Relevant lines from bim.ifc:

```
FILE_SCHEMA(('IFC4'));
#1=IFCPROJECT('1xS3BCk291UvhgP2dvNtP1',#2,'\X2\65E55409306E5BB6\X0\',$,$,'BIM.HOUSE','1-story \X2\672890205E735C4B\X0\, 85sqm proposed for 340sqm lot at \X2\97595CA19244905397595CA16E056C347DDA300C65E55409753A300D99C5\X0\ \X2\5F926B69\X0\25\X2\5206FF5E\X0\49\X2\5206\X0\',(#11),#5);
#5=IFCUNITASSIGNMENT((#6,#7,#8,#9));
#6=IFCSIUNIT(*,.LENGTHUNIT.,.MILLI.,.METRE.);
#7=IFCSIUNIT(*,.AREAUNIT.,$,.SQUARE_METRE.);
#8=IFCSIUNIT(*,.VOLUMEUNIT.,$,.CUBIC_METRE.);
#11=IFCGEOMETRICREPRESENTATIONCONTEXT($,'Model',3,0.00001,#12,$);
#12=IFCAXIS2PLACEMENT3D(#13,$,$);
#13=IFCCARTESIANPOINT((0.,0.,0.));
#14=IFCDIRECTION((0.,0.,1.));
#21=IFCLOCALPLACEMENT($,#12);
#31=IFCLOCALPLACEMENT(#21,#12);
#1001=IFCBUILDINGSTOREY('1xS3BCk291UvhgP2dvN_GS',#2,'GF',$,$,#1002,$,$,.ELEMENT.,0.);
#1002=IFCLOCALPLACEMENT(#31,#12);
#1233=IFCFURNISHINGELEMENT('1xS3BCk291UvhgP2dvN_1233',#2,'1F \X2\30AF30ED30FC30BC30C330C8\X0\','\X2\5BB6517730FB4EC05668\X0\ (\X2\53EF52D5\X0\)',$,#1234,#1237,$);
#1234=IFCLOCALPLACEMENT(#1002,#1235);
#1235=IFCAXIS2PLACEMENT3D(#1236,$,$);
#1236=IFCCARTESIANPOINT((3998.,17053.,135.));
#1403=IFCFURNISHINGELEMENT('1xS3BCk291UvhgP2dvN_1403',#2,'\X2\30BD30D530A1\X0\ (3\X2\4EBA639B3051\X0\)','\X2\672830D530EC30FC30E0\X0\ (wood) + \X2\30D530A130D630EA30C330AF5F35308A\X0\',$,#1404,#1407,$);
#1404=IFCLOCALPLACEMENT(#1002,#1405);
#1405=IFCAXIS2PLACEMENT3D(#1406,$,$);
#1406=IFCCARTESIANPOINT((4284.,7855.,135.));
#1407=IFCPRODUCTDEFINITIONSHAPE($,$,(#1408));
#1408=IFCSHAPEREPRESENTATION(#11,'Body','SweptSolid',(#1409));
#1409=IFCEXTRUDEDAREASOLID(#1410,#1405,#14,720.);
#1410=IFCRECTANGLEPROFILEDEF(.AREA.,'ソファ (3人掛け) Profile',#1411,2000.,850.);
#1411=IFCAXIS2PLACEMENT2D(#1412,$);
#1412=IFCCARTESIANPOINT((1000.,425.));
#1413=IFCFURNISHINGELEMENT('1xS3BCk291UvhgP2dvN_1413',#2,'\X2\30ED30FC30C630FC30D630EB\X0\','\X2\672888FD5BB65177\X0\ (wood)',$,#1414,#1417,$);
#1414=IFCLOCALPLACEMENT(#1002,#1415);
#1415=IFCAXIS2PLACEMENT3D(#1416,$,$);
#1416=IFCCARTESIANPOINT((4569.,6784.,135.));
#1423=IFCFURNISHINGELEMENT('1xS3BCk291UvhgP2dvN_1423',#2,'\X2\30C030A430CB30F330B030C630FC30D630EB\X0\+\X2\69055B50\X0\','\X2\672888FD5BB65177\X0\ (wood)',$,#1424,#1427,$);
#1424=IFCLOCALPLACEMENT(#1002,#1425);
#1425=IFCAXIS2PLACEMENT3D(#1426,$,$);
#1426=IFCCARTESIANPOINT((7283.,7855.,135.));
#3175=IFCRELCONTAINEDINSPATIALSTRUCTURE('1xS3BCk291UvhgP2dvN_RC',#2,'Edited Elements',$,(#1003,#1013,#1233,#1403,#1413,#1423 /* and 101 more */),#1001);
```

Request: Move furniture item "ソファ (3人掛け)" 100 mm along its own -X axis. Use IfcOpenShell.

```python
import ifcopenshell
import ifcopenshell.api.geometry
import ifcopenshell.util.placement
import ifcopenshell.util.unit

model = ifcopenshell.open("bim.ifc")
unit_scale = ifcopenshell.util.unit.calculate_unit_scale(model)

item = model.by_guid("1xS3BCk291UvhgP2dvN_1403")
matrix = ifcopenshell.util.placement.get_local_placement(item.ObjectPlacement)
matrix[:3, 3] -= matrix[:3, 0] * 0.1 / unit_scale
ifcopenshell.api.geometry.edit_object_placement(model, product=item, matrix=matrix, is_si=False)

print(ifcopenshell.util.placement.get_local_placement(item.ObjectPlacement).round(3) + 0.0)

model.write("bim_rev.ifc")
```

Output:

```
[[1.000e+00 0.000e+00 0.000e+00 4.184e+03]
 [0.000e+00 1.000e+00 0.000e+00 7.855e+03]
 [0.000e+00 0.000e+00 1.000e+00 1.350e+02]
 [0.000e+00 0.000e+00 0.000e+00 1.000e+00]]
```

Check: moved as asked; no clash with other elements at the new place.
